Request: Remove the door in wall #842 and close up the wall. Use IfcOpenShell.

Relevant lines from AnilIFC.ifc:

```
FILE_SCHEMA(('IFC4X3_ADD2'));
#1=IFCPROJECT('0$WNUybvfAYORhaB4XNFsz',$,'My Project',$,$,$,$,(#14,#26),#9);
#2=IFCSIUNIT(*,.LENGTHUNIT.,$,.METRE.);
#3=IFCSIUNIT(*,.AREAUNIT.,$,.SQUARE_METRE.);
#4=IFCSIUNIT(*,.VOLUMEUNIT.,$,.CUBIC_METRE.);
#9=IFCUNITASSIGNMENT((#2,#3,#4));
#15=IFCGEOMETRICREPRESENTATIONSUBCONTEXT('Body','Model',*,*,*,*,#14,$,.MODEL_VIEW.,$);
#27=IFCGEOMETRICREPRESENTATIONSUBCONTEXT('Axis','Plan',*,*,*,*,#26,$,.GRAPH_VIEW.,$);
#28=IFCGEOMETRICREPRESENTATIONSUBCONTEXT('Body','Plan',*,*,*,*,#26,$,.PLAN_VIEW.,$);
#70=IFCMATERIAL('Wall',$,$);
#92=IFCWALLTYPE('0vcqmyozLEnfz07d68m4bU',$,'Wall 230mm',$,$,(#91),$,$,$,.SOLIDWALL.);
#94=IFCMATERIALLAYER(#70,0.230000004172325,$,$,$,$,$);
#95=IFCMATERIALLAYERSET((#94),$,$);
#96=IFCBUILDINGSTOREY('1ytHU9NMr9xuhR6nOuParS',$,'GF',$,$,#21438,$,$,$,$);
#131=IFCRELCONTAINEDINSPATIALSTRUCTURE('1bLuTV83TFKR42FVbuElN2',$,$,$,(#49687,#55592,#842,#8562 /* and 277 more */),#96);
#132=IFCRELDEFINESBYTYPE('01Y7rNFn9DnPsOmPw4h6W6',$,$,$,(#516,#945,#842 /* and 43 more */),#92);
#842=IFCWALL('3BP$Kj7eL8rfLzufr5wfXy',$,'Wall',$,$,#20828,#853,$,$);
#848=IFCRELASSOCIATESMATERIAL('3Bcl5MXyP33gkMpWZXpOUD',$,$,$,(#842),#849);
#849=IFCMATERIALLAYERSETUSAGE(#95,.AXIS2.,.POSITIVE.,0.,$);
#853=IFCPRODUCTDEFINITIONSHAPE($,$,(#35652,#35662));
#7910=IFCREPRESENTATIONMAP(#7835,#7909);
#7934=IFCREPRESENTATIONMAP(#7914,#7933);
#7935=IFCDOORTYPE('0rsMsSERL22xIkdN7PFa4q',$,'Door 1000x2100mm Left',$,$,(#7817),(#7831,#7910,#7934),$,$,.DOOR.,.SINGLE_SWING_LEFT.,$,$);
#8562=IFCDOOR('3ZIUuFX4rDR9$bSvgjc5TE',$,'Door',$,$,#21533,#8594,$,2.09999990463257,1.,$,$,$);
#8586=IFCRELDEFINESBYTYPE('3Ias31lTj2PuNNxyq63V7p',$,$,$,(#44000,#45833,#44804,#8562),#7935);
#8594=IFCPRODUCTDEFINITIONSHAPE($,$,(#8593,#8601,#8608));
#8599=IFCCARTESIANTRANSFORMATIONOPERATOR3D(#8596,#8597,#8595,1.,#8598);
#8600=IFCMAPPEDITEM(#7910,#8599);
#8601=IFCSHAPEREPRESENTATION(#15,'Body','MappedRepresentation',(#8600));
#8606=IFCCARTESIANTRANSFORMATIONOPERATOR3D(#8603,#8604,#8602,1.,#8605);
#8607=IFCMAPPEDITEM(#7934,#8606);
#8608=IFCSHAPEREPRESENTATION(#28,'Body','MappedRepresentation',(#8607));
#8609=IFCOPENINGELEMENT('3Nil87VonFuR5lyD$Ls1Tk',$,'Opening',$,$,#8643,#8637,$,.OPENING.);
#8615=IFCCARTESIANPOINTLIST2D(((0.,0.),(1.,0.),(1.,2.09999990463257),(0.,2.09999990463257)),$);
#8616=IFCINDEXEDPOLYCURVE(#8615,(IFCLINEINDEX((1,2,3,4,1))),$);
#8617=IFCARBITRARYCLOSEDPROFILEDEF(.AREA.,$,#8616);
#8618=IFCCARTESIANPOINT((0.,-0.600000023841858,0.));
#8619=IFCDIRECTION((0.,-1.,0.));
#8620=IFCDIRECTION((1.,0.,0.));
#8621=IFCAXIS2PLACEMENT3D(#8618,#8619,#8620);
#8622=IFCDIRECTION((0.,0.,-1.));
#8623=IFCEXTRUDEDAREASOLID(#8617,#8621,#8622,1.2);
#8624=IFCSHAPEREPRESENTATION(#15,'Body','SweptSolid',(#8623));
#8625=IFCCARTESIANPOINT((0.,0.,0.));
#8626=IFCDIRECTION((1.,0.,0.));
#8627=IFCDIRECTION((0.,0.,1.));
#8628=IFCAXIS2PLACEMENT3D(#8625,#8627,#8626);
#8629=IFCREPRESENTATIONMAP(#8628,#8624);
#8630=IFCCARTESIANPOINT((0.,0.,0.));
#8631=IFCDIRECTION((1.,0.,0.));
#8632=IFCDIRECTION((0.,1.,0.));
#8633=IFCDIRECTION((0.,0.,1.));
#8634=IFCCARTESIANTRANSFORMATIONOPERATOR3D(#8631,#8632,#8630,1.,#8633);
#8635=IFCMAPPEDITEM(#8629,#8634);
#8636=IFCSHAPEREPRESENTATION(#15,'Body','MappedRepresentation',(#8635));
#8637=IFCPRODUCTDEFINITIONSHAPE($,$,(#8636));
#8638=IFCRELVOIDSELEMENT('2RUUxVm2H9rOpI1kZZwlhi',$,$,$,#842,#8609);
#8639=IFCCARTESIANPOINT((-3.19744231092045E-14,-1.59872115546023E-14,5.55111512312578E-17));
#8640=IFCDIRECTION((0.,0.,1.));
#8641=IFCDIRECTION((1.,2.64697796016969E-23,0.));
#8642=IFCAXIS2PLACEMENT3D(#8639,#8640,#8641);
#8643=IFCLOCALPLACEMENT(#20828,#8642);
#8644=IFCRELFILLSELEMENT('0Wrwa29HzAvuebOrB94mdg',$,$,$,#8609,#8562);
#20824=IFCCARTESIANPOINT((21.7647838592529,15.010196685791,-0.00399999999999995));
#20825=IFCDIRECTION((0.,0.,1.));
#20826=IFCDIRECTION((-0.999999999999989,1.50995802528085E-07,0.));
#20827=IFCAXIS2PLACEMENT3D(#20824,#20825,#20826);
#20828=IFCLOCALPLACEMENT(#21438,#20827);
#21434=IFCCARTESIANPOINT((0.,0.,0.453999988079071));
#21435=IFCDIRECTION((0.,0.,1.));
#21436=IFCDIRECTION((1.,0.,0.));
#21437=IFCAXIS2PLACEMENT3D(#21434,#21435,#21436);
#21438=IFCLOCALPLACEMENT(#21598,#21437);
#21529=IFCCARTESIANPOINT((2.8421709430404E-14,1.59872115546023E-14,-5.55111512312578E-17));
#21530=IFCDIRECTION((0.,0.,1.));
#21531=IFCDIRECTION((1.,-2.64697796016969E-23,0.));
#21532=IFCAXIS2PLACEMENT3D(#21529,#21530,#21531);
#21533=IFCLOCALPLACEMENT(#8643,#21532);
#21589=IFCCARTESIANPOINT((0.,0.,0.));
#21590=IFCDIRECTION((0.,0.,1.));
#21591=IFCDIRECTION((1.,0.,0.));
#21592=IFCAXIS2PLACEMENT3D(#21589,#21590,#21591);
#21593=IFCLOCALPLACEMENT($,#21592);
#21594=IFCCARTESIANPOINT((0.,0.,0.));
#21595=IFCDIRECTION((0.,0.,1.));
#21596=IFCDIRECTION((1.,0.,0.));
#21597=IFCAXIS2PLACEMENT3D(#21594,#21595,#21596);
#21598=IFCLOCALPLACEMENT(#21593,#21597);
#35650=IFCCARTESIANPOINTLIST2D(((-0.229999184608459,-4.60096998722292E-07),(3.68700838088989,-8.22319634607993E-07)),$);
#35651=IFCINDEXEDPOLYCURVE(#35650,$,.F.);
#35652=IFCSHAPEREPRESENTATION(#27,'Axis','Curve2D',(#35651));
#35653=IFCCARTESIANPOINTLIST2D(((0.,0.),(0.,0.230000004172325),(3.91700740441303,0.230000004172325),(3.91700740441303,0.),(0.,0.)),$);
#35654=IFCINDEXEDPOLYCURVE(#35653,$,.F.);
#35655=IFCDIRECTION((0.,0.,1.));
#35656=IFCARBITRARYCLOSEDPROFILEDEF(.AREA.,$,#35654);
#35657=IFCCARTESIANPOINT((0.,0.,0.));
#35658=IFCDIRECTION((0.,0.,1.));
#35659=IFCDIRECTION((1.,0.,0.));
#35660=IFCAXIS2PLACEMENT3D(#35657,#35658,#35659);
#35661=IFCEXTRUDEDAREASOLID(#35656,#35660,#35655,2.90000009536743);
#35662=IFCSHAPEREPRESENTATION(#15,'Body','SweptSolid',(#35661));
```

```python
import ifcopenshell
import ifcopenshell.api.feature
import ifcopenshell.api.root
import ifcopenshell.geom
import ifcopenshell.util.shape

model = ifcopenshell.open("AnilIFC.ifc")
settings = ifcopenshell.geom.settings()


def volume(element):
    """Net volume in cubic metres, openings subtracted."""
    shape = ifcopenshell.geom.create_shape(settings, element)
    return ifcopenshell.util.shape.get_volume(shape.geometry)


door = model.by_id(8562)
opening = door.FillsVoids[0].RelatingOpeningElement
wall = opening.VoidsElements[0].RelatingBuildingElement
before = volume(wall)

ifcopenshell.api.root.remove_product(model, product=door)
ifcopenshell.api.feature.remove_feature(model, feature=opening)

after = volume(wall)

print(f"wall volume {before:.3f} -> {after:.3f} m3")

model.write("AnilIFC_edited.ifc")
```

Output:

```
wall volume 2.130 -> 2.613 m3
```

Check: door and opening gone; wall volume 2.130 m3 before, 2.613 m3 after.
